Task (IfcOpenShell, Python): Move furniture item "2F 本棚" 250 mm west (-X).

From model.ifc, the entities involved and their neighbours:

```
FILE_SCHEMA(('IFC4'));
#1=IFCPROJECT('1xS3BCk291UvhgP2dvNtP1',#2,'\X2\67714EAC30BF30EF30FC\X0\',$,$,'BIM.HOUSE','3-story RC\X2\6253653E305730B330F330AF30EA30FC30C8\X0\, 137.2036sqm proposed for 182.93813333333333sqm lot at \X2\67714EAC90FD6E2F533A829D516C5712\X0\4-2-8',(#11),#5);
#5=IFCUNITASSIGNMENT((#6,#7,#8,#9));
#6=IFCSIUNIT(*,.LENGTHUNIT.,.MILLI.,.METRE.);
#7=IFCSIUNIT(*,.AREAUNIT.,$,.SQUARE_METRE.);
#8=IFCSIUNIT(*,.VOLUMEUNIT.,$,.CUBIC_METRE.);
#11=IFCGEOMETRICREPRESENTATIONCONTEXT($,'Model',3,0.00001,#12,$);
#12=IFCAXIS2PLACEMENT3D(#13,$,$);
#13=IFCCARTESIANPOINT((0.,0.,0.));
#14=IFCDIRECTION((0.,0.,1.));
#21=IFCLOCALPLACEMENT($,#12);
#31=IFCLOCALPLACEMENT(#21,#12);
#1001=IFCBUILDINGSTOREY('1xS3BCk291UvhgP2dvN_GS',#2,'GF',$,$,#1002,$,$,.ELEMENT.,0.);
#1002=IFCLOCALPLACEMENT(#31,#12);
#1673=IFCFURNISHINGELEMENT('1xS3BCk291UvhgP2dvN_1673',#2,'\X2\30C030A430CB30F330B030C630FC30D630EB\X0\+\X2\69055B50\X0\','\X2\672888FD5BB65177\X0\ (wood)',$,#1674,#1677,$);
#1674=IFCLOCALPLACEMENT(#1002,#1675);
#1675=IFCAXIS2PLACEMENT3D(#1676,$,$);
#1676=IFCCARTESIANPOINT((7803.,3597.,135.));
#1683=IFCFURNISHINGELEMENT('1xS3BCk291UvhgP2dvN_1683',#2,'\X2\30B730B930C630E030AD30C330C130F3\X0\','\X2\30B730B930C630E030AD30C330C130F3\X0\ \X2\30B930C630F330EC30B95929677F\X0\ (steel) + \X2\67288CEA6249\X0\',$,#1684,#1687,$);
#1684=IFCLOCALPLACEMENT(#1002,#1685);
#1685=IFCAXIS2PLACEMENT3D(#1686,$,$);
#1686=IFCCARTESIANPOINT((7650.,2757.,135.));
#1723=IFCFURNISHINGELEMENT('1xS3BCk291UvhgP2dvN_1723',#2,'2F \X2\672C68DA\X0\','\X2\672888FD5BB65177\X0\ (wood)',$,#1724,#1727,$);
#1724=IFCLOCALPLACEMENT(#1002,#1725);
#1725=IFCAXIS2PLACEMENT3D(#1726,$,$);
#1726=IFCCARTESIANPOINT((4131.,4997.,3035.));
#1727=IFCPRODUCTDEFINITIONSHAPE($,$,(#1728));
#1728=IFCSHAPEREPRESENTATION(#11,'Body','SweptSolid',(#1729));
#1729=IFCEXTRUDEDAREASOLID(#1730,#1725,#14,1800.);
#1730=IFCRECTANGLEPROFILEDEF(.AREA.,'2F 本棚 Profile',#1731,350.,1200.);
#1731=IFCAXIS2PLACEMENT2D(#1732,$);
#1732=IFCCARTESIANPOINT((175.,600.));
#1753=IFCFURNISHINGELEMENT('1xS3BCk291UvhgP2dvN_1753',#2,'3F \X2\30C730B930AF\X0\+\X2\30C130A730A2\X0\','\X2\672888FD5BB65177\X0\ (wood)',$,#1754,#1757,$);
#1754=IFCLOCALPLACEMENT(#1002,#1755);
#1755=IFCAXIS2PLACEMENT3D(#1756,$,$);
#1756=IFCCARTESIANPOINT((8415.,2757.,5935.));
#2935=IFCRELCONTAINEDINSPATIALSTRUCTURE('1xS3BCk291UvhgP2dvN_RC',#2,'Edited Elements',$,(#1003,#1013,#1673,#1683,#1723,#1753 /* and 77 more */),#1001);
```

```python
import ifcopenshell
import ifcopenshell.api.geometry
import ifcopenshell.util.placement

model = ifcopenshell.open("model.ifc")

item = model.by_guid("1xS3BCk291UvhgP2dvN_1723")
matrix = ifcopenshell.util.placement.get_local_placement(item.ObjectPlacement)
matrix[0, 3] -= 250.0
ifcopenshell.api.geometry.edit_object_placement(model, product=item, matrix=matrix, is_si=False)

print(ifcopenshell.util.placement.get_local_placement(item.ObjectPlacement).round(3) + 0.0)

model.write("model_v2.ifc")
```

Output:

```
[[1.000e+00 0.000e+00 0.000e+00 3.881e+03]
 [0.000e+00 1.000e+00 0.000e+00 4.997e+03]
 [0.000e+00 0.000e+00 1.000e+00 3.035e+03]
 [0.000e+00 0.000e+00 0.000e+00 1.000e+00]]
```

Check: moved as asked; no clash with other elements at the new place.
